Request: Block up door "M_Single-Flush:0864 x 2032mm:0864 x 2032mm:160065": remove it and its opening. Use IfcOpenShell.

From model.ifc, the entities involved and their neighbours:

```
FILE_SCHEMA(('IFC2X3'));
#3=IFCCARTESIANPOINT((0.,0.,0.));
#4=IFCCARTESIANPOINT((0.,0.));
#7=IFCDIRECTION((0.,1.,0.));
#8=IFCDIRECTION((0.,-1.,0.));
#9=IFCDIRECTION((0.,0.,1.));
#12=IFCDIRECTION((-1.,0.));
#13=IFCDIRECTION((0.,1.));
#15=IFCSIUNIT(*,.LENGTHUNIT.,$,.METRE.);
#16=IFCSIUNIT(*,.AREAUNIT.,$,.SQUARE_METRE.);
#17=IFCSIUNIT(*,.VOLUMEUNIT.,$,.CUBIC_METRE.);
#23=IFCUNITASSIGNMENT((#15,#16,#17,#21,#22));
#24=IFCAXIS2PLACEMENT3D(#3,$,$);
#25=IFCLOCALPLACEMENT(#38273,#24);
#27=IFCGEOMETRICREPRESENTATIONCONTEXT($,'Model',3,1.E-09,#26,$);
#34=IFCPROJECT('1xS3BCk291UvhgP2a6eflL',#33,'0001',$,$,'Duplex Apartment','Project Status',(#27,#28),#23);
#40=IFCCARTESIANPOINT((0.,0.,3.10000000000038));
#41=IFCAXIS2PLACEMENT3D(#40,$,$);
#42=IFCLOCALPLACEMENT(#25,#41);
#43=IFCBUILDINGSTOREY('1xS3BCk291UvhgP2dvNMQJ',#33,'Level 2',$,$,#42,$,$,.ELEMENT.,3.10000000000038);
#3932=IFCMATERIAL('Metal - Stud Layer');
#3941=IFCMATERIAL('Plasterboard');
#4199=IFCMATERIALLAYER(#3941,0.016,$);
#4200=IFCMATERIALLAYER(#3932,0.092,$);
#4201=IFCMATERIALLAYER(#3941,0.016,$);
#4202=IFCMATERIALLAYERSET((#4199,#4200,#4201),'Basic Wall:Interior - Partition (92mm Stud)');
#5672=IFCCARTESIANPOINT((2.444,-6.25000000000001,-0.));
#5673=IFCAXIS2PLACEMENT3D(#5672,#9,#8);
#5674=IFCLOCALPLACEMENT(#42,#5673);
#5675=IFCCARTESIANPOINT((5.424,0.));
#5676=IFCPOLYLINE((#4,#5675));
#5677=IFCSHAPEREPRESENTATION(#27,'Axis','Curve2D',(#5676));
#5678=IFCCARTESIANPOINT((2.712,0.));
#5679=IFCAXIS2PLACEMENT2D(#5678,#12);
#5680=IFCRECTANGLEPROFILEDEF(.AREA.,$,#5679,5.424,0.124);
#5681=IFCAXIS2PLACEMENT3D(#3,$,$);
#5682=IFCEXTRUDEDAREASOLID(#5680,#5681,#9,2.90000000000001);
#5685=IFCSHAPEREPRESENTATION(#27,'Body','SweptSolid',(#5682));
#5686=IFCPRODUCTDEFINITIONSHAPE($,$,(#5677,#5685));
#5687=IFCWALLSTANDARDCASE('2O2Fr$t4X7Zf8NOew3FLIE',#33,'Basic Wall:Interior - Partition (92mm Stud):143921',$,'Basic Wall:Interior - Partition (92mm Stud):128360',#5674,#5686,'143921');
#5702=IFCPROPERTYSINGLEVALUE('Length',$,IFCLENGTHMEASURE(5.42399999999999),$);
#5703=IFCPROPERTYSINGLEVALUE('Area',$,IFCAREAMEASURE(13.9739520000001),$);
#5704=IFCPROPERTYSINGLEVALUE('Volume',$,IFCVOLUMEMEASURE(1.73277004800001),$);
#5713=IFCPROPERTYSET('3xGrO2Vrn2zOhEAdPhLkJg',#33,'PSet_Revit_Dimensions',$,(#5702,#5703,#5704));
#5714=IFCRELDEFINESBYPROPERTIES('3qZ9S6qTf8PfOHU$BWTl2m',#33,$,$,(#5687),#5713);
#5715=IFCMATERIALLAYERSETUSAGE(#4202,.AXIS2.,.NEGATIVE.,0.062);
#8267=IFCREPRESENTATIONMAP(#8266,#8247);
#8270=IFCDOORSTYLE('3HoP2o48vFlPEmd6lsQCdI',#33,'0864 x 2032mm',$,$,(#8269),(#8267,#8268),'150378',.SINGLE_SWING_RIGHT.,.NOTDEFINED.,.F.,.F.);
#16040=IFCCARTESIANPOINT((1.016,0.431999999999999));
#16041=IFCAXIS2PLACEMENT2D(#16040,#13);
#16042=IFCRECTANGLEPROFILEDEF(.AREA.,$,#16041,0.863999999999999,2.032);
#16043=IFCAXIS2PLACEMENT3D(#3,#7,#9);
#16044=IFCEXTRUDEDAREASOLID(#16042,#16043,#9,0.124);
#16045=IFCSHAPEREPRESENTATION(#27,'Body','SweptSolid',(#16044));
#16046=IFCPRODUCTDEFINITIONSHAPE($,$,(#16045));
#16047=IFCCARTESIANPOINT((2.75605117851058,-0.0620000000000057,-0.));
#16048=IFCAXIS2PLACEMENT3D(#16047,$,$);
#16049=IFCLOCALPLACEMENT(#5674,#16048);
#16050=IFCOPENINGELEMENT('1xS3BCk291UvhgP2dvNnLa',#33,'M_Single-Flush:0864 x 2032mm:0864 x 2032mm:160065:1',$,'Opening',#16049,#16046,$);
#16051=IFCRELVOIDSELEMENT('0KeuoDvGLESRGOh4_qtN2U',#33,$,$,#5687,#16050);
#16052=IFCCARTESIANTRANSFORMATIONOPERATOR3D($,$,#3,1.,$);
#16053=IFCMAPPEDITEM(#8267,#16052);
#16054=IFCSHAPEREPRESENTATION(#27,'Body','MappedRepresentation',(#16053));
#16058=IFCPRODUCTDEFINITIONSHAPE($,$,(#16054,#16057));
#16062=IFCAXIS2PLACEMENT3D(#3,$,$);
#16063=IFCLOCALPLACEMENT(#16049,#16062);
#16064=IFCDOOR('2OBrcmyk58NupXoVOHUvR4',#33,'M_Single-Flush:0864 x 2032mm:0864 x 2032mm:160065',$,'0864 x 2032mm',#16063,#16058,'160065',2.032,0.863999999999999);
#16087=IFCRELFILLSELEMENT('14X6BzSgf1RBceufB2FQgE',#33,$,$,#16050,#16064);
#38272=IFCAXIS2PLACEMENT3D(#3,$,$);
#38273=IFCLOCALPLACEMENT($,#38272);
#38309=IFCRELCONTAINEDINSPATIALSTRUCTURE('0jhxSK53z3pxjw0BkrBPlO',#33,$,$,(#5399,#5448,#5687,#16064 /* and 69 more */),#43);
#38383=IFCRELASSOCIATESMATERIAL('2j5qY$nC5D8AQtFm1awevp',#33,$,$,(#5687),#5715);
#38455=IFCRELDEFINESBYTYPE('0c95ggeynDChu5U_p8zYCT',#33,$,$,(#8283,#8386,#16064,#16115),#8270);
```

```python
import ifcopenshell
import ifcopenshell.api.feature
import ifcopenshell.api.pset
import ifcopenshell.api.root
import ifcopenshell.geom
import ifcopenshell.util.element
import ifcopenshell.util.shape
import ifcopenshell.util.unit

model = ifcopenshell.open("model.ifc")
area_scale = ifcopenshell.util.unit.calculate_unit_scale(model, "AREAUNIT")
volume_scale = ifcopenshell.util.unit.calculate_unit_scale(model, "VOLUMEUNIT")
settings = ifcopenshell.geom.settings()


def volume(element):
    """Net volume in cubic metres, openings subtracted."""
    shape = ifcopenshell.geom.create_shape(settings, element)
    return ifcopenshell.util.shape.get_volume(shape.geometry)


door = model.by_guid("2OBrcmyk58NupXoVOHUvR4")
opening = door.FillsVoids[0].RelatingOpeningElement
wall = opening.VoidsElements[0].RelatingBuildingElement
before = volume(wall)

ifcopenshell.api.root.remove_product(model, product=door)
ifcopenshell.api.feature.remove_feature(model, feature=opening)

after = volume(wall)
thickness = 0.124  # wall thickness in metres

# Update the wall's stored quantities.
pset = model.by_id(ifcopenshell.util.element.get_pset(wall, "PSet_Revit_Dimensions", should_inherit=False)["id"])
ifcopenshell.api.pset.edit_pset(model, pset=pset, properties={
    "Area": model.create_entity("IfcAreaMeasure", after / thickness / area_scale),
    "Volume": model.create_entity("IfcVolumeMeasure", after / volume_scale),
})

print(f"wall volume {before:.3f} -> {after:.3f} m3")

model.write("model-out.ifc")
```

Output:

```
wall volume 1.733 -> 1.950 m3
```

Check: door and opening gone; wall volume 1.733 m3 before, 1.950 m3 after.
